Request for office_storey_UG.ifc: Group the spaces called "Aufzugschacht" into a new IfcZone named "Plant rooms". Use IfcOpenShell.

First a look at what the model holds.

```python
import ifcopenshell

model = ifcopenshell.open("office_storey_UG.ifc")
print(model.schema)
seen = {}
for space in model.by_type("IfcSpace"):
    seen[space.LongName] = seen.get(space.LongName, 0) + 1
for name, count in sorted(seen.items(), key=str):
    print(count, "x", name)
print("zones:", [z.Name for z in model.by_type("IfcZone")][:20])
```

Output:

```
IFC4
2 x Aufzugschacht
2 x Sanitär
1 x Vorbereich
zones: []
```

```python
import ifcopenshell
import ifcopenshell.api.group
import ifcopenshell.api.root

model = ifcopenshell.open("office_storey_UG.ifc")

names = {"Aufzugschacht"}
spaces = [s for s in model.by_type("IfcSpace") if s.LongName in names]

zone = ifcopenshell.api.root.create_entity(model, ifc_class="IfcZone", name="Plant rooms")
ifcopenshell.api.group.assign_group(model, products=spaces, group=zone)
print(len(spaces), "spaces in", zone.Name)

model.write("office_storey_UG_edited.ifc")
```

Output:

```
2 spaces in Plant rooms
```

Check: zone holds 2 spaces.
